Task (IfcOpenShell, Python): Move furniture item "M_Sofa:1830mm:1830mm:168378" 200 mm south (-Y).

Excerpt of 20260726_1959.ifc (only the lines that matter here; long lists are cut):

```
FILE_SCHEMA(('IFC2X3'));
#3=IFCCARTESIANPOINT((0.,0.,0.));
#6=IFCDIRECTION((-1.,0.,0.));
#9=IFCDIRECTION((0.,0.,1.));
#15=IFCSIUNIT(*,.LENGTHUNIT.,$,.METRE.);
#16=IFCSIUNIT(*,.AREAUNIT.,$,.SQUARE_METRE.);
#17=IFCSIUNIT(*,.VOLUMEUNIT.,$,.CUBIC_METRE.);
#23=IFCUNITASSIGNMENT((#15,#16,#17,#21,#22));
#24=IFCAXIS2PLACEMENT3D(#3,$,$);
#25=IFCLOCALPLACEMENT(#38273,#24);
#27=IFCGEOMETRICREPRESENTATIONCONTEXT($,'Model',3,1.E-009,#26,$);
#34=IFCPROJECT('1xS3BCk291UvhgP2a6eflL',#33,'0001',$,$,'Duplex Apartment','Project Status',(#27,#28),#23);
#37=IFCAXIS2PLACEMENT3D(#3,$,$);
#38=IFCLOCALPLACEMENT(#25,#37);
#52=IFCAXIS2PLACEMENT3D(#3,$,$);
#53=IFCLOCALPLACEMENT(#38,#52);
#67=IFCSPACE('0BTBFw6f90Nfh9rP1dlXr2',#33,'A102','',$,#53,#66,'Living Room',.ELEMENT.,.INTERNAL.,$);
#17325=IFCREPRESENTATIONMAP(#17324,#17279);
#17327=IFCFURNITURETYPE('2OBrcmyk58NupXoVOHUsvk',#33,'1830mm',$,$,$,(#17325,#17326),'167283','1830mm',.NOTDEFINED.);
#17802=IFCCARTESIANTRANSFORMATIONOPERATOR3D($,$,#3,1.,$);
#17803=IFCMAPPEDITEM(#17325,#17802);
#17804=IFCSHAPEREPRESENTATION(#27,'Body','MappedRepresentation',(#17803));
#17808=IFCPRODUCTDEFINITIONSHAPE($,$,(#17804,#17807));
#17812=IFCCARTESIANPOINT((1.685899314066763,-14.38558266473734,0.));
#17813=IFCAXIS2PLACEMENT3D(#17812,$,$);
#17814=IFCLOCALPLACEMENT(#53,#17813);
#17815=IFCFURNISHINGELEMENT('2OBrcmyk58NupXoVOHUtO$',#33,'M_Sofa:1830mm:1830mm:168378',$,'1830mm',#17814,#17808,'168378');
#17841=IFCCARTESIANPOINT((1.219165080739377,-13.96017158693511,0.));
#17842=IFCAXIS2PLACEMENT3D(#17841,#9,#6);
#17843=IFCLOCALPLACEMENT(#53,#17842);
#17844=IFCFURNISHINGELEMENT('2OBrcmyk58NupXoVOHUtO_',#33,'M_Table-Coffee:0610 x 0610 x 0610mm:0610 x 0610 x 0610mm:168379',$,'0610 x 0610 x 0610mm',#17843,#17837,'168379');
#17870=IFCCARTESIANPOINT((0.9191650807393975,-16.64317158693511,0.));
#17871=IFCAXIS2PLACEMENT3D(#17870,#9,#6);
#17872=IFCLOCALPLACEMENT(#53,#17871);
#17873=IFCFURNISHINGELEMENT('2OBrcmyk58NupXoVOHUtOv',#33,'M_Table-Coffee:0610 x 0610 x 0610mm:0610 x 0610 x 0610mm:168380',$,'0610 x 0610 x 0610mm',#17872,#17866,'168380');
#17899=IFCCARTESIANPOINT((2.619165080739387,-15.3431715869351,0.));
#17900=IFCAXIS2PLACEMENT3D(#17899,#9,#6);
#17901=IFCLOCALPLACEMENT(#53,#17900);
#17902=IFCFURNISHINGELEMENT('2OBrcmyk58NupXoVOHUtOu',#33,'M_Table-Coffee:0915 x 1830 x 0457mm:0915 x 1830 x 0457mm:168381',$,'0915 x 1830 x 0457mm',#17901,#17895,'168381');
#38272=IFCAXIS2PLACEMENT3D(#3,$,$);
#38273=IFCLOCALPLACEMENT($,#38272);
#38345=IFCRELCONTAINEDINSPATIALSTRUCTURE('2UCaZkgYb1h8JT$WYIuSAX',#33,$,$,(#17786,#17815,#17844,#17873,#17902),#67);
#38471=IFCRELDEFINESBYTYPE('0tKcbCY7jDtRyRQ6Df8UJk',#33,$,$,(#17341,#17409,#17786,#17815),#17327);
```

```python
import ifcopenshell
import ifcopenshell.api.geometry
import ifcopenshell.util.placement
import ifcopenshell.util.unit

model = ifcopenshell.open("20260726_1959.ifc")
unit_scale = ifcopenshell.util.unit.calculate_unit_scale(model)

item = model.by_guid("2OBrcmyk58NupXoVOHUtO$")
matrix = ifcopenshell.util.placement.get_local_placement(item.ObjectPlacement)
matrix[1, 3] -= 0.2 / unit_scale
ifcopenshell.api.geometry.edit_object_placement(model, product=item, matrix=matrix, is_si=False)

print(ifcopenshell.util.placement.get_local_placement(item.ObjectPlacement).round(3) + 0.0)

model.write("20260726_1959_v2.ifc")
```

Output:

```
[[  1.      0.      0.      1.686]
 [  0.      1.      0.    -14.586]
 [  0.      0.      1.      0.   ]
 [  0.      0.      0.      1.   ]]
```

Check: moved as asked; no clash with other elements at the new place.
